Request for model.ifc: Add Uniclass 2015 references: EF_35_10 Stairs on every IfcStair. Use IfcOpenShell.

First a look at what the model holds.

```python
import ifcopenshell

model = ifcopenshell.open("model.ifc")
print(model.schema)
print("classifications:", [c.Name for c in model.by_type("IfcClassification")])
for ifc_class in ("IfcDoor", "IfcRoof", "IfcStair", "IfcWall", "IfcWindow"):
    print(ifc_class, len(model.by_type(ifc_class)))
```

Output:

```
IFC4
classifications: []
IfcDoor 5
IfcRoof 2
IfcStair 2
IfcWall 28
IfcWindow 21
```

```python
import ifcopenshell
import ifcopenshell.api.classification

model = ifcopenshell.open("model.ifc")

system = ifcopenshell.api.classification.add_classification(model, classification="Uniclass 2015")

codes = {
    "IfcStair": ("EF_35_10", "Stairs"),
}
for ifc_class, (code, name) in codes.items():
    products = model.by_type(ifc_class)
    ifcopenshell.api.classification.add_reference(
        model, products=products, classification=system, identification=code, name=name
    )
    print(code, len(products))

model.write("model_edited.ifc")
```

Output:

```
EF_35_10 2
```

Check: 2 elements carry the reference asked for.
